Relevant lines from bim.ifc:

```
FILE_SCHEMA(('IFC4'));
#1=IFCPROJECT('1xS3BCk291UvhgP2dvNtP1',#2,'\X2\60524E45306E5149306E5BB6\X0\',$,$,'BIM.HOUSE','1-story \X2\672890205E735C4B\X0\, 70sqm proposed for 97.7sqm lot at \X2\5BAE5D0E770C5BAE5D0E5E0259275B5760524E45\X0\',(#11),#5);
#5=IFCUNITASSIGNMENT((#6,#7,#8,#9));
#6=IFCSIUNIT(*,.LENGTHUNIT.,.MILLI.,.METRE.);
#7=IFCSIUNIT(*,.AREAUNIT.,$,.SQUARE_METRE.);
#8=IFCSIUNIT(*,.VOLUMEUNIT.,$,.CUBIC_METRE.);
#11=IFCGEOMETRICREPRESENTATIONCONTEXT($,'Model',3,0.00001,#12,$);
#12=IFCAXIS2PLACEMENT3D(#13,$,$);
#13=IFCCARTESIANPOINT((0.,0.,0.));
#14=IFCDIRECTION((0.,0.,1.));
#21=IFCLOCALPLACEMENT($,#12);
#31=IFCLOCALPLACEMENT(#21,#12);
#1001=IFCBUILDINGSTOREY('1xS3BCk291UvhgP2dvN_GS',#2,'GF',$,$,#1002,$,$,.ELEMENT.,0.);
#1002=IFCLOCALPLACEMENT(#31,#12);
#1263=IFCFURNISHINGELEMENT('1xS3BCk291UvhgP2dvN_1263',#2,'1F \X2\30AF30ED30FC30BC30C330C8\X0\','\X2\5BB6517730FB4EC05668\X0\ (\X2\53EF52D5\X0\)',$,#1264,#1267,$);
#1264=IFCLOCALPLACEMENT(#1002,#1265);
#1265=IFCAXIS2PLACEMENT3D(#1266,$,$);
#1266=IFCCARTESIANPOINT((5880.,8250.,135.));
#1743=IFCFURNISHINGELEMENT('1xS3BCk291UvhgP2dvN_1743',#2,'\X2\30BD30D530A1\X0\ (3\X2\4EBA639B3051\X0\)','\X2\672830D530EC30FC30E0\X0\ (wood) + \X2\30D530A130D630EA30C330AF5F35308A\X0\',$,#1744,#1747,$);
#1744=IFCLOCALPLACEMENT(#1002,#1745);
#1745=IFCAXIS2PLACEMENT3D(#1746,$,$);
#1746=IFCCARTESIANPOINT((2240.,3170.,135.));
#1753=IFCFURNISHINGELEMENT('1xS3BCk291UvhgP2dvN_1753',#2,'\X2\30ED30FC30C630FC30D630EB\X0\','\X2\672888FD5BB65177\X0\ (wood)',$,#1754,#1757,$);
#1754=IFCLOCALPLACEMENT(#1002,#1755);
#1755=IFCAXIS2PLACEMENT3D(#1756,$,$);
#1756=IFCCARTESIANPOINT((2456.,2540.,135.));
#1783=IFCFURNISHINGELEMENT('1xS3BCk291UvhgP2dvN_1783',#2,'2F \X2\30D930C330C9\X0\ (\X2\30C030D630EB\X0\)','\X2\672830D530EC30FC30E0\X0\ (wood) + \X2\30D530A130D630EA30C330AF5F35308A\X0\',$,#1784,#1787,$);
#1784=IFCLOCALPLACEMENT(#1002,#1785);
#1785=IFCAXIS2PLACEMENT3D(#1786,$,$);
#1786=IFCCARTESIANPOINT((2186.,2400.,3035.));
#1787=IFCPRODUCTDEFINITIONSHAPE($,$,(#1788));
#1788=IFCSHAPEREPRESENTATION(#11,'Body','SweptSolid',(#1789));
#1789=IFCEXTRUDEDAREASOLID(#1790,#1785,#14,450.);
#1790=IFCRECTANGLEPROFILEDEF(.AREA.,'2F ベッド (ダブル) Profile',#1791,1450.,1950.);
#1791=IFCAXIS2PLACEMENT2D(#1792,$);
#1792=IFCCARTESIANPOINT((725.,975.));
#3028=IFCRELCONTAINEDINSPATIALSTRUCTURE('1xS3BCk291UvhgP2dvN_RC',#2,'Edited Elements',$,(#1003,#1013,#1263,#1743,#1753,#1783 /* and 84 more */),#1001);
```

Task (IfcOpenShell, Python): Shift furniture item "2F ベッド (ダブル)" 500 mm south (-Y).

```python
import ifcopenshell
import ifcopenshell.api.geometry
import ifcopenshell.util.placement

model = ifcopenshell.open("bim.ifc")

item = model.by_guid("1xS3BCk291UvhgP2dvN_1783")
matrix = ifcopenshell.util.placement.get_local_placement(item.ObjectPlacement)
matrix[1, 3] -= 500.0
ifcopenshell.api.geometry.edit_object_placement(model, product=item, matrix=matrix, is_si=False)

print(ifcopenshell.util.placement.get_local_placement(item.ObjectPlacement).round(3) + 0.0)

model.write("bim_rev.ifc")
```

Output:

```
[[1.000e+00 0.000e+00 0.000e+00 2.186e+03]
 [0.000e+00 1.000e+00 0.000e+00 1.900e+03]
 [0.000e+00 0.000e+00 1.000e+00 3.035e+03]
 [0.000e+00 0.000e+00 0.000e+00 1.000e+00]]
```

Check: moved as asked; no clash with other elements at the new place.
